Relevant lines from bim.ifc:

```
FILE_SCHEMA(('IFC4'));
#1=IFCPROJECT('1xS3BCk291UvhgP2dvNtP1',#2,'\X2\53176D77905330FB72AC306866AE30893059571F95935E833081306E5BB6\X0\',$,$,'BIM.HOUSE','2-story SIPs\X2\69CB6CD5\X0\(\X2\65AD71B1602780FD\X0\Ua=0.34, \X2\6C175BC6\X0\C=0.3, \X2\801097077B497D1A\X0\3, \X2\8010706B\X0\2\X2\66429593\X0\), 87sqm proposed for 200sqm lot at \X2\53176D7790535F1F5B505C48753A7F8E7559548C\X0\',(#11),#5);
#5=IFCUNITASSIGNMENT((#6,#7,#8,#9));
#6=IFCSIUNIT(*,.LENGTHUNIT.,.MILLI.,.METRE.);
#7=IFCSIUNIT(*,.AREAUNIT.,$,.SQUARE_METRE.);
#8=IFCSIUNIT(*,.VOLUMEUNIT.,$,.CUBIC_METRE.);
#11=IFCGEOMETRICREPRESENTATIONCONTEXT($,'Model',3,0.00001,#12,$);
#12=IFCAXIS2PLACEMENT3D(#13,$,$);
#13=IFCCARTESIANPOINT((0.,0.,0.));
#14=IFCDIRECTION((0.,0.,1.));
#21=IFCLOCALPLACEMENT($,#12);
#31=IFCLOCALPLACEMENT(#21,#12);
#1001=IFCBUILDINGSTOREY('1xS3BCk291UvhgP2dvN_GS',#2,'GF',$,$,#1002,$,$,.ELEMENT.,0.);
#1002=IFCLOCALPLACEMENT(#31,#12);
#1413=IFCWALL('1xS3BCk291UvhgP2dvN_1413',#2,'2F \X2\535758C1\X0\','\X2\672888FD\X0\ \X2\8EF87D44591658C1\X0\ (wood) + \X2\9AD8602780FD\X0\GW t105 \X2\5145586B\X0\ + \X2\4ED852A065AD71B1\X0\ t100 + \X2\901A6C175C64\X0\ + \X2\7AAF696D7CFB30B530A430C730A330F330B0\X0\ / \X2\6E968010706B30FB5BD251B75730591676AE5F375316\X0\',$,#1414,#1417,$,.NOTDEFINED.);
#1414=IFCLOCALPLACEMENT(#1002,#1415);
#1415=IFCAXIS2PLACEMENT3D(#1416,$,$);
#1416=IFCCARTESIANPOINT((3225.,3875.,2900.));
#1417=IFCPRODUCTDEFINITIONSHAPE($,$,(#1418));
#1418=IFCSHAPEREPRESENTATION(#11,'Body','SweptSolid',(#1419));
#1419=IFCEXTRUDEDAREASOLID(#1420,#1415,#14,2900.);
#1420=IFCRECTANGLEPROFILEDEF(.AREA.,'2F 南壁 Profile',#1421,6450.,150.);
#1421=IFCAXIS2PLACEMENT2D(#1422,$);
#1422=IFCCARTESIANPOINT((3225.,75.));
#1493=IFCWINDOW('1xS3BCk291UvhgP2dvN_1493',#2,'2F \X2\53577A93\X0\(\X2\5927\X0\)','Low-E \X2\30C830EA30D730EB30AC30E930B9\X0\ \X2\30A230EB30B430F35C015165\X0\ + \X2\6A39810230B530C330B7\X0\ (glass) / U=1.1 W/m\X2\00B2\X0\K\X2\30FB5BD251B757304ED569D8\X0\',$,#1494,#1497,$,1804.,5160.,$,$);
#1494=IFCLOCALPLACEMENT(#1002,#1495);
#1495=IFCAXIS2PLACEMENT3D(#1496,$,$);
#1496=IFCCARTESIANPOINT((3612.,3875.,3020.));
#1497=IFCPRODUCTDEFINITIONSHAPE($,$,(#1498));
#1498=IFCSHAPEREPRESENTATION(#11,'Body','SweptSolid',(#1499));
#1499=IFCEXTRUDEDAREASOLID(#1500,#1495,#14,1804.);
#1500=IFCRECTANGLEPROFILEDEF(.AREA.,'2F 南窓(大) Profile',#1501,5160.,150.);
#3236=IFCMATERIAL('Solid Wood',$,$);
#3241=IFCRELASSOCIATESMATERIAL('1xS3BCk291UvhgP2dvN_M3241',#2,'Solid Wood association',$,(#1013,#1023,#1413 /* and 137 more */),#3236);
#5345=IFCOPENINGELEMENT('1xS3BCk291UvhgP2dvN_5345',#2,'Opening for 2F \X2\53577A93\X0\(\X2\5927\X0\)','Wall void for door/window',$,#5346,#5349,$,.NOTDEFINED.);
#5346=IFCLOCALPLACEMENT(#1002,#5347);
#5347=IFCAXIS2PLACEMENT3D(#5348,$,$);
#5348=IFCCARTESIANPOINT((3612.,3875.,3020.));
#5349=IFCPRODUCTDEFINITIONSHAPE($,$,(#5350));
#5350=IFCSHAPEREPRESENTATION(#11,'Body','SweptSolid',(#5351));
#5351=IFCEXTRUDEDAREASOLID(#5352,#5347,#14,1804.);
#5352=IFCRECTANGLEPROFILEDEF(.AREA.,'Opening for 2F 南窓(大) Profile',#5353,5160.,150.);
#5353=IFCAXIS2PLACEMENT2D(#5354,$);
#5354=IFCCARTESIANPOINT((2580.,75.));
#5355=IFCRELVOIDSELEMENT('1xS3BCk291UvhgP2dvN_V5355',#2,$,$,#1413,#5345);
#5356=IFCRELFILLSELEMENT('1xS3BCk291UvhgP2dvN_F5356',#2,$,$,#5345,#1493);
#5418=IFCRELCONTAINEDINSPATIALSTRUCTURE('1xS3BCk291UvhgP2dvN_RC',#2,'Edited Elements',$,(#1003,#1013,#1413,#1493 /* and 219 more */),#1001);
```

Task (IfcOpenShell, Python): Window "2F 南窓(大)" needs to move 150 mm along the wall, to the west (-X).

```python
import ifcopenshell
import ifcopenshell.api.geometry
import ifcopenshell.util.placement
import ifcopenshell.util.unit

model = ifcopenshell.open("bim.ifc")
unit_scale = ifcopenshell.util.unit.calculate_unit_scale(model)

window = model.by_id(1493)
opening = window.FillsVoids[0].RelatingOpeningElement
wall = opening.VoidsElements[0].RelatingBuildingElement

wall_matrix = ifcopenshell.util.placement.get_local_placement(wall.ObjectPlacement)
shift = wall_matrix[:3, 0] * -0.15 / unit_scale
before = ifcopenshell.util.placement.get_local_placement(window.ObjectPlacement)[:3, 3].copy()

# The window is not placed relative to its opening, so move both.
for product in (opening, window):
    matrix = ifcopenshell.util.placement.get_local_placement(product.ObjectPlacement)
    matrix[:3, 3] += shift
    ifcopenshell.api.geometry.edit_object_placement(model, product=product, matrix=matrix, is_si=False)

after = ifcopenshell.util.placement.get_local_placement(window.ObjectPlacement)[:3, 3]
print("window moved by", (after - before).round(3) + 0.0)

model.write("bim_updated.ifc")
```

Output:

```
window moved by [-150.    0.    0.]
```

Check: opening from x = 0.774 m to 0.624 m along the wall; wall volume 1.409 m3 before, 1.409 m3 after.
